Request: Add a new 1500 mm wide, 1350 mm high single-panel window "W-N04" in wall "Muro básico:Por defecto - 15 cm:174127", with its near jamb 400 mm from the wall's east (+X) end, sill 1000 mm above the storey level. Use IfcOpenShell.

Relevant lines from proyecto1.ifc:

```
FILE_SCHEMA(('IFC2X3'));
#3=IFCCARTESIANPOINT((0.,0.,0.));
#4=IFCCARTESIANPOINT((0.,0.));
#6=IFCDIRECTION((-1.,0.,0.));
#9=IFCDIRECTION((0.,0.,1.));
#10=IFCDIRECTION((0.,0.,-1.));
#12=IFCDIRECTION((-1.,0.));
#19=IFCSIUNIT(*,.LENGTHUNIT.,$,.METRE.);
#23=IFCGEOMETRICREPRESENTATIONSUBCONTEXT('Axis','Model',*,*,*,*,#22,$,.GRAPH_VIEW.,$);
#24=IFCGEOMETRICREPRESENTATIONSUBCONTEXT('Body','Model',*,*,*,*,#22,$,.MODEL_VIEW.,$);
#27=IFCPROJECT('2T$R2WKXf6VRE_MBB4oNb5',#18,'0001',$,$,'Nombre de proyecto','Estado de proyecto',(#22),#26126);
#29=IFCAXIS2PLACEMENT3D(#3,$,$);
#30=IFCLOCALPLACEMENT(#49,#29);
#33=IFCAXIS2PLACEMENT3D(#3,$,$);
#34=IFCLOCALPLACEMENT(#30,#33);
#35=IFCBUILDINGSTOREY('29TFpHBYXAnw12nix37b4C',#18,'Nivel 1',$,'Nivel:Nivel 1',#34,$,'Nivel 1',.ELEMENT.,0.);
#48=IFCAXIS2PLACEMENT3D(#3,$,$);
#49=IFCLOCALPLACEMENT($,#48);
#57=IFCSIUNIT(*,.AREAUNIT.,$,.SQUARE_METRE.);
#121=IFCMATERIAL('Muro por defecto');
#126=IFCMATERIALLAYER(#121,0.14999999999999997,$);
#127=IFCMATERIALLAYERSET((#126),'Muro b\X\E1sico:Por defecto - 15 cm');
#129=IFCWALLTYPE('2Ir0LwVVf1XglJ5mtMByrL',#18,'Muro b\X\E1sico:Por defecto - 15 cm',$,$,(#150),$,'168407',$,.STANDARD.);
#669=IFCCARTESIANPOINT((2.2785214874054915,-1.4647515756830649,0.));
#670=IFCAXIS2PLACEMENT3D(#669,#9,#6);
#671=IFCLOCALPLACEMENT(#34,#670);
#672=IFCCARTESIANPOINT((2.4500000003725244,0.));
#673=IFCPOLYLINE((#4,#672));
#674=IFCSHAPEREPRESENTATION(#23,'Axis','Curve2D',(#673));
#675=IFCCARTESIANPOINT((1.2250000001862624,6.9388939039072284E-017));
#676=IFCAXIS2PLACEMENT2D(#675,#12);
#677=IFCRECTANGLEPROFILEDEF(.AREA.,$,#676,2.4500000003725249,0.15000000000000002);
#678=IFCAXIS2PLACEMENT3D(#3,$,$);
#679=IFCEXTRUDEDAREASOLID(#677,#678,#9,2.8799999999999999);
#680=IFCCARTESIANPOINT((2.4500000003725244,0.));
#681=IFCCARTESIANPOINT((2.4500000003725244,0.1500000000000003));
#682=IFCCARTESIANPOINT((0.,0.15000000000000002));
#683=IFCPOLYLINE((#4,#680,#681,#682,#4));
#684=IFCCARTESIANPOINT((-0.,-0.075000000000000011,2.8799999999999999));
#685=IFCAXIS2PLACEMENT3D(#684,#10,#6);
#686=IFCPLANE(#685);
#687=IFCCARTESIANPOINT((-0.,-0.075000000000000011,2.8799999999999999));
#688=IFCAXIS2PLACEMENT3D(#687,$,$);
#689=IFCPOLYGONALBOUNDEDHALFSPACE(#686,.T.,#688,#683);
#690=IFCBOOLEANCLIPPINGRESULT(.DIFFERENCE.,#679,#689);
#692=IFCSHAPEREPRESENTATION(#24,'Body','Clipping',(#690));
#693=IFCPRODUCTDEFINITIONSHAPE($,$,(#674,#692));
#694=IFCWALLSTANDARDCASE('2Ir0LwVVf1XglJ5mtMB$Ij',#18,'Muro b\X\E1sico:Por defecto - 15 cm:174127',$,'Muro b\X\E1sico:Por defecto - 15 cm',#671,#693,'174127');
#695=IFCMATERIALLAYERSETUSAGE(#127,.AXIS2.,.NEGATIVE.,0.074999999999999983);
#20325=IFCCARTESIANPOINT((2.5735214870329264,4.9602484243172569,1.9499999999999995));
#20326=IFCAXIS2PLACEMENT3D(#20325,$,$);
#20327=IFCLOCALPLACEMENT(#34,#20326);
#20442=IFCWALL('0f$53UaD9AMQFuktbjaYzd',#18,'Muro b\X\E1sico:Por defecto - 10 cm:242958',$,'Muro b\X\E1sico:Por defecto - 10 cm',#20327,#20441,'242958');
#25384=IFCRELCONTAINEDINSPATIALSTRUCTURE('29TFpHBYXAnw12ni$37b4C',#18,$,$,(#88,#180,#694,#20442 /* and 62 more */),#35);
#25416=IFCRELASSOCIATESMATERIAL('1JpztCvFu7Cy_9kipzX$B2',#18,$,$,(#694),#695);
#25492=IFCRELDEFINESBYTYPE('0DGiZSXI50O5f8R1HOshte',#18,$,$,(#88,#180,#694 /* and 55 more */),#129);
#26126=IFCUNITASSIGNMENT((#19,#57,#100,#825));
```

```python
import numpy as np
import ifcopenshell
import ifcopenshell.api.feature
import ifcopenshell.api.geometry
import ifcopenshell.api.root
import ifcopenshell.api.spatial
import ifcopenshell.api.type
import ifcopenshell.geom
import ifcopenshell.util.element
import ifcopenshell.util.placement
import ifcopenshell.util.representation
import ifcopenshell.util.shape
import ifcopenshell.util.unit

model = ifcopenshell.open("proyecto1.ifc")
unit_scale = ifcopenshell.util.unit.calculate_unit_scale(model)
settings = ifcopenshell.geom.settings()


def volume(element):
    """Net volume in cubic metres, openings subtracted."""
    shape = ifcopenshell.geom.create_shape(settings, element)
    return ifcopenshell.util.shape.get_volume(shape.geometry)


wall = model.by_id(694)
storey = ifcopenshell.util.element.get_container(wall, ifc_class="IfcBuildingStorey")
context = ifcopenshell.util.representation.get_context(model, "Model", "Body", "MODEL_VIEW")
before = volume(wall)

width, height, from_end, sill = 1.5, 1.35, 0.4, 1  # metres

# The wall runs along its own X axis, and the end named is its -X end.
wall_shape = ifcopenshell.geom.create_shape(settings, wall)
x, y, z = ifcopenshell.util.shape.get_vertices(wall_shape.geometry).T
start = x.min() + from_end
face, thickness = float(y.min()), float(y.max() - y.min())
wall_matrix = ifcopenshell.util.placement.get_local_placement(wall.ObjectPlacement)
level = ifcopenshell.util.placement.get_local_placement(storey.ObjectPlacement)[2, 3]


def in_wall(x, y):
    """Placement at x, y metres in the wall's axes, at sill height."""
    matrix = wall_matrix.copy()
    matrix[:, 3] = wall_matrix @ np.array([x / unit_scale, y / unit_scale, 0.0, 1.0])
    matrix[2, 3] = level + sill / unit_scale
    return matrix


# Opening: a box that overshoots both wall faces by 50 mm.
opening = ifcopenshell.api.root.create_entity(model, ifc_class="IfcOpeningElement")
box = ifcopenshell.api.geometry.add_wall_representation(
    model, context=context, length=width, height=height, thickness=thickness + 0.1
)
ifcopenshell.api.geometry.assign_representation(model, product=opening, representation=box)
ifcopenshell.api.geometry.edit_object_placement(model, product=opening, matrix=in_wall(start, face - 0.05), is_si=False)
ifcopenshell.api.feature.add_feature(model, feature=opening, element=wall)

window = ifcopenshell.api.root.create_entity(model, ifc_class="IfcWindow", name="W-N04")
window.OverallWidth, window.OverallHeight = width / unit_scale, height / unit_scale
body = ifcopenshell.api.geometry.add_window_representation(
    model,
    context=context,
    overall_width=window.OverallWidth,
    overall_height=window.OverallHeight,
    partition_type="SINGLE_PANEL",
)
ifcopenshell.api.geometry.assign_representation(model, product=window, representation=body)
ifcopenshell.api.spatial.assign_container(model, products=[window], relating_structure=storey)
fills = ifcopenshell.api.feature.add_filling(model, opening=opening, element=window)
fills.OwnerHistory = window.OwnerHistory  # required in IFC2X3

# IFC2X3 keeps the operation on the window style.
style = ifcopenshell.api.root.create_entity(model, ifc_class="IfcWindowStyle", name="W-N04")
style.OperationType, style.ConstructionType = "SINGLE_PANEL", "NOTDEFINED"
style.ParameterTakesPrecedence = style.Sizeable = False
ifcopenshell.api.type.assign_type(model, related_objects=[window], relating_type=style)

# Centre the window in the wall's thickness.
ifcopenshell.api.geometry.edit_object_placement(model, product=window, matrix=in_wall(start, face), is_si=False)
window_shape = ifcopenshell.geom.create_shape(settings, window)
depth = ifcopenshell.util.shape.get_vertices(window_shape.geometry)[:, 1]
offset = face + thickness / 2 - (depth.min() + depth.max()) / 2
ifcopenshell.api.geometry.edit_object_placement(model, product=window, matrix=in_wall(start, offset), is_si=False)

after = volume(wall)

print(f"wall volume {before:.3f} -> {after:.3f} m3")

model.write("proyecto1-out.ifc")
```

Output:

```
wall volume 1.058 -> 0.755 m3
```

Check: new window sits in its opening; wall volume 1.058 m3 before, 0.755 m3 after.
